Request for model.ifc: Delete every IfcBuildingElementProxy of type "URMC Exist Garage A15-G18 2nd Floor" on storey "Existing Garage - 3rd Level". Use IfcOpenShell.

First a look at what the model holds.

```python
import ifcopenshell
import ifcopenshell.util.element

model = ifcopenshell.open("model.ifc")
print(model.schema)
storey = next(s for s in model.by_type("IfcBuildingStorey") if s.Name == "Existing Garage - 3rd Level")
proxies = [e for e in ifcopenshell.util.element.get_decomposition(storey) if e.is_a("IfcBuildingElementProxy")]
seen = {}
for e in proxies:
    element_type = ifcopenshell.util.element.get_type(e)
    name = element_type.Name if element_type not in (None, e) else None
    seen[name] = seen.get(name, 0) + 1
for name, count in sorted(seen.items(), key=str):
    print(count, "x", name)
```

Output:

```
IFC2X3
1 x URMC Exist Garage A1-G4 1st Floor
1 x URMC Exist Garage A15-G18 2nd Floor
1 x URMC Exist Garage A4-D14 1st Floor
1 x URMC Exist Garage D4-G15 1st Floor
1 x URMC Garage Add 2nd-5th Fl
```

```python
import ifcopenshell
import ifcopenshell.api.root
import ifcopenshell.util.element

model = ifcopenshell.open("model.ifc")

storey = next(s for s in model.by_type("IfcBuildingStorey") if s.Name == "Existing Garage - 3rd Level")
proxies = [e for e in ifcopenshell.util.element.get_decomposition(storey) if e.is_a("IfcBuildingElementProxy")]
targets = [e for e in proxies if (t := ifcopenshell.util.element.get_type(e)) not in (None, e) and t.Name == "URMC Exist Garage A15-G18 2nd Floor"]

for e in targets:
    ifcopenshell.api.root.remove_product(model, product=e)
print(len(targets), "removed")

model.write("model_rev.ifc")
```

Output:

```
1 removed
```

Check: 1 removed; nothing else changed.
